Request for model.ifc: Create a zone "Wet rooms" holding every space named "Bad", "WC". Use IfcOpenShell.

First a look at what the model holds.

```python
import ifcopenshell

model = ifcopenshell.open("model.ifc")
print(model.schema)
seen = {}
for space in model.by_type("IfcSpace"):
    seen[space.LongName] = seen.get(space.LongName, 0) + 1
for name, count in sorted(seen.items(), key=str):
    print(count, "x", name)
print("zones:", [z.Name for z in model.by_type("IfcZone")][:20])
```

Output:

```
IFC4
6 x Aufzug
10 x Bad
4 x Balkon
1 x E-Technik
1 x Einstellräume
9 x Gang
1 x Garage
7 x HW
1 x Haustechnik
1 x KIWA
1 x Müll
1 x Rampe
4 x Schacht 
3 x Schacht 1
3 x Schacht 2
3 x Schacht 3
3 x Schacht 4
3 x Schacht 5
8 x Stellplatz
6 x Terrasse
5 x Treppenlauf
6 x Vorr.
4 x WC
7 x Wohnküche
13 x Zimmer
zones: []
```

```python
import ifcopenshell
import ifcopenshell.api.group
import ifcopenshell.api.root

model = ifcopenshell.open("model.ifc")

names = {"Bad", "WC"}
spaces = [s for s in model.by_type("IfcSpace") if s.LongName in names]

zone = ifcopenshell.api.root.create_entity(model, ifc_class="IfcZone", name="Wet rooms")
ifcopenshell.api.group.assign_group(model, products=spaces, group=zone)
print(len(spaces), "spaces in", zone.Name)

model.write("model_updated.ifc")
```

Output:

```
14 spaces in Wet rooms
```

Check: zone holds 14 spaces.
